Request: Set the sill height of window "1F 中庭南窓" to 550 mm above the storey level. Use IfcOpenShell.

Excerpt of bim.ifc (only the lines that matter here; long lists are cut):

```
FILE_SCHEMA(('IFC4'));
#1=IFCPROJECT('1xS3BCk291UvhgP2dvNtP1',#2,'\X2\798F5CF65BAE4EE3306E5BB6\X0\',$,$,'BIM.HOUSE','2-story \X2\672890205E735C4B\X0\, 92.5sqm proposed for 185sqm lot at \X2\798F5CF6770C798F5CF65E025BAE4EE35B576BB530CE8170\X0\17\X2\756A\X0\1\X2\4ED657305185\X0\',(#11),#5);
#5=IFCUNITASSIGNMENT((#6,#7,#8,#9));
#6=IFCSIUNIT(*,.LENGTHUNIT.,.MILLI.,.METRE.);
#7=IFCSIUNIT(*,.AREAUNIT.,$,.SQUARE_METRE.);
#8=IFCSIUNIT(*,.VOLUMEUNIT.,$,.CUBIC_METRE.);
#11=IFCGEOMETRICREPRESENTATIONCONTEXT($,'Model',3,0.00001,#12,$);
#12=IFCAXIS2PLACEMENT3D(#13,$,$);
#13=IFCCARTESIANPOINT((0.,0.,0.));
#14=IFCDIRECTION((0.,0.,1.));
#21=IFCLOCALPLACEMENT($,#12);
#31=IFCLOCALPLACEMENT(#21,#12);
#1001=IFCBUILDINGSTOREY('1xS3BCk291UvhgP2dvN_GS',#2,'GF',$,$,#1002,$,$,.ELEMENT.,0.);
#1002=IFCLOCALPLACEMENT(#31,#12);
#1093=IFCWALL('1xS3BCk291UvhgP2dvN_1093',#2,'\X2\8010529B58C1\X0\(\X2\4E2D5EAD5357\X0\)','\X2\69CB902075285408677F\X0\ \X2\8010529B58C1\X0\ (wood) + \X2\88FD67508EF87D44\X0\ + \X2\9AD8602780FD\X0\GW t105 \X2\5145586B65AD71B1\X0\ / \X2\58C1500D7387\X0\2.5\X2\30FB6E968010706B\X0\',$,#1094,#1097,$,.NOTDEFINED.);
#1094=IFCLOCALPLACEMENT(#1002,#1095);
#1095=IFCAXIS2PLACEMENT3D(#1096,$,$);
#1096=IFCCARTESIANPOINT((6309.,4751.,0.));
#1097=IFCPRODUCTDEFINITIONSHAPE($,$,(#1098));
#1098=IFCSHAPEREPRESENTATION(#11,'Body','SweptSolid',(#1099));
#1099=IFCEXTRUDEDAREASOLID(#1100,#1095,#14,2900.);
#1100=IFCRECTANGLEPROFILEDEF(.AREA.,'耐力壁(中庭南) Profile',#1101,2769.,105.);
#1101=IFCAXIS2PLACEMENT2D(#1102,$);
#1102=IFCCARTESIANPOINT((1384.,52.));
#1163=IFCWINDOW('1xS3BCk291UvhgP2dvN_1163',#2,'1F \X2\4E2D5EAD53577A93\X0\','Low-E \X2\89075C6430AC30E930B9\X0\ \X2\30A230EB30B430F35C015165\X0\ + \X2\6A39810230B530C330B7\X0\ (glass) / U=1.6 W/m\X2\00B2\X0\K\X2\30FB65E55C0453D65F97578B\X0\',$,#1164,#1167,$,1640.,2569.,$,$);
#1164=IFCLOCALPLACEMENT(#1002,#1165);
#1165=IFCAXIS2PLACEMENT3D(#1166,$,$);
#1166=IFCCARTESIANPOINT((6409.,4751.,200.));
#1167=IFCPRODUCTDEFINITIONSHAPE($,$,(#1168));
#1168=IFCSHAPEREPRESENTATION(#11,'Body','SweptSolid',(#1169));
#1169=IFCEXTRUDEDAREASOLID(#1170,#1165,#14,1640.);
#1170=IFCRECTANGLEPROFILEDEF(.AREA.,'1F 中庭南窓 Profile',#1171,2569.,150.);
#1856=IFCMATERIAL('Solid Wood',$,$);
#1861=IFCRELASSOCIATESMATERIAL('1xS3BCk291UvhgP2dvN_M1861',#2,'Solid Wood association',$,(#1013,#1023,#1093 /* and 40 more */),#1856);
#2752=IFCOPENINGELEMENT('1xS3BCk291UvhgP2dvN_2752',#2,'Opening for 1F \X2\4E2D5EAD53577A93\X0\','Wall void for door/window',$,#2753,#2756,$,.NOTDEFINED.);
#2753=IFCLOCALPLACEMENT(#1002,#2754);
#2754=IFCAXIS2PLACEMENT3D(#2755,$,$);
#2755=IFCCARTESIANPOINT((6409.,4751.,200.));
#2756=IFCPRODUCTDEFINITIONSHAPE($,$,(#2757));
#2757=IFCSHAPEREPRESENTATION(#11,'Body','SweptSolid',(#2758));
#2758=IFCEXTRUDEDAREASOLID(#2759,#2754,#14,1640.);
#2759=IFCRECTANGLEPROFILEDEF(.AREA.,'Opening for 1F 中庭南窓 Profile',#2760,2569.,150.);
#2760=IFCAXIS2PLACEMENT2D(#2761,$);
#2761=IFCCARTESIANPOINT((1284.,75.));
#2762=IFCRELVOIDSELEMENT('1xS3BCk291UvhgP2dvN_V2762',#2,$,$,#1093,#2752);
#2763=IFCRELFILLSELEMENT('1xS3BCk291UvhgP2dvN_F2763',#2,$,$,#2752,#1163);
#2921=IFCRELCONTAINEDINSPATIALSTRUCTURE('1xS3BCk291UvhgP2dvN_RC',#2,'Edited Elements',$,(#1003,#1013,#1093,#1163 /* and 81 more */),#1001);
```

```python
import numpy as np
import ifcopenshell
import ifcopenshell.api.geometry
import ifcopenshell.geom
import ifcopenshell.util.element
import ifcopenshell.util.placement
import ifcopenshell.util.shape
import ifcopenshell.util.unit

model = ifcopenshell.open("bim.ifc")
unit_scale = ifcopenshell.util.unit.calculate_unit_scale(model)

window = model.by_guid("1xS3BCk291UvhgP2dvN_1163")
opening = window.FillsVoids[0].RelatingOpeningElement
storey = ifcopenshell.util.element.get_container(window, ifc_class="IfcBuildingStorey")
level = ifcopenshell.util.placement.get_local_placement(storey.ObjectPlacement)[2, 3]

# The opening's origin need not be at the sill, so measure its lowest point.
shape = ifcopenshell.geom.create_shape(ifcopenshell.geom.settings(), opening)
bottom = ifcopenshell.util.shape.get_shape_bottom_elevation(shape, shape.geometry) / unit_scale
dz = level + 550.0 - bottom

shift = np.array([0.0, 0.0, dz])
# The window is not placed relative to its opening, so move both.
for product in (opening, window):
    matrix = ifcopenshell.util.placement.get_local_placement(product.ObjectPlacement)
    matrix[:3, 3] += shift
    ifcopenshell.api.geometry.edit_object_placement(model, product=product, matrix=matrix, is_si=False)

print(f"moved by {dz * unit_scale:+.3f} m")

model.write("bim-out.ifc")
```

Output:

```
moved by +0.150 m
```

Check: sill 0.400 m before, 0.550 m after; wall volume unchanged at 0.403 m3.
